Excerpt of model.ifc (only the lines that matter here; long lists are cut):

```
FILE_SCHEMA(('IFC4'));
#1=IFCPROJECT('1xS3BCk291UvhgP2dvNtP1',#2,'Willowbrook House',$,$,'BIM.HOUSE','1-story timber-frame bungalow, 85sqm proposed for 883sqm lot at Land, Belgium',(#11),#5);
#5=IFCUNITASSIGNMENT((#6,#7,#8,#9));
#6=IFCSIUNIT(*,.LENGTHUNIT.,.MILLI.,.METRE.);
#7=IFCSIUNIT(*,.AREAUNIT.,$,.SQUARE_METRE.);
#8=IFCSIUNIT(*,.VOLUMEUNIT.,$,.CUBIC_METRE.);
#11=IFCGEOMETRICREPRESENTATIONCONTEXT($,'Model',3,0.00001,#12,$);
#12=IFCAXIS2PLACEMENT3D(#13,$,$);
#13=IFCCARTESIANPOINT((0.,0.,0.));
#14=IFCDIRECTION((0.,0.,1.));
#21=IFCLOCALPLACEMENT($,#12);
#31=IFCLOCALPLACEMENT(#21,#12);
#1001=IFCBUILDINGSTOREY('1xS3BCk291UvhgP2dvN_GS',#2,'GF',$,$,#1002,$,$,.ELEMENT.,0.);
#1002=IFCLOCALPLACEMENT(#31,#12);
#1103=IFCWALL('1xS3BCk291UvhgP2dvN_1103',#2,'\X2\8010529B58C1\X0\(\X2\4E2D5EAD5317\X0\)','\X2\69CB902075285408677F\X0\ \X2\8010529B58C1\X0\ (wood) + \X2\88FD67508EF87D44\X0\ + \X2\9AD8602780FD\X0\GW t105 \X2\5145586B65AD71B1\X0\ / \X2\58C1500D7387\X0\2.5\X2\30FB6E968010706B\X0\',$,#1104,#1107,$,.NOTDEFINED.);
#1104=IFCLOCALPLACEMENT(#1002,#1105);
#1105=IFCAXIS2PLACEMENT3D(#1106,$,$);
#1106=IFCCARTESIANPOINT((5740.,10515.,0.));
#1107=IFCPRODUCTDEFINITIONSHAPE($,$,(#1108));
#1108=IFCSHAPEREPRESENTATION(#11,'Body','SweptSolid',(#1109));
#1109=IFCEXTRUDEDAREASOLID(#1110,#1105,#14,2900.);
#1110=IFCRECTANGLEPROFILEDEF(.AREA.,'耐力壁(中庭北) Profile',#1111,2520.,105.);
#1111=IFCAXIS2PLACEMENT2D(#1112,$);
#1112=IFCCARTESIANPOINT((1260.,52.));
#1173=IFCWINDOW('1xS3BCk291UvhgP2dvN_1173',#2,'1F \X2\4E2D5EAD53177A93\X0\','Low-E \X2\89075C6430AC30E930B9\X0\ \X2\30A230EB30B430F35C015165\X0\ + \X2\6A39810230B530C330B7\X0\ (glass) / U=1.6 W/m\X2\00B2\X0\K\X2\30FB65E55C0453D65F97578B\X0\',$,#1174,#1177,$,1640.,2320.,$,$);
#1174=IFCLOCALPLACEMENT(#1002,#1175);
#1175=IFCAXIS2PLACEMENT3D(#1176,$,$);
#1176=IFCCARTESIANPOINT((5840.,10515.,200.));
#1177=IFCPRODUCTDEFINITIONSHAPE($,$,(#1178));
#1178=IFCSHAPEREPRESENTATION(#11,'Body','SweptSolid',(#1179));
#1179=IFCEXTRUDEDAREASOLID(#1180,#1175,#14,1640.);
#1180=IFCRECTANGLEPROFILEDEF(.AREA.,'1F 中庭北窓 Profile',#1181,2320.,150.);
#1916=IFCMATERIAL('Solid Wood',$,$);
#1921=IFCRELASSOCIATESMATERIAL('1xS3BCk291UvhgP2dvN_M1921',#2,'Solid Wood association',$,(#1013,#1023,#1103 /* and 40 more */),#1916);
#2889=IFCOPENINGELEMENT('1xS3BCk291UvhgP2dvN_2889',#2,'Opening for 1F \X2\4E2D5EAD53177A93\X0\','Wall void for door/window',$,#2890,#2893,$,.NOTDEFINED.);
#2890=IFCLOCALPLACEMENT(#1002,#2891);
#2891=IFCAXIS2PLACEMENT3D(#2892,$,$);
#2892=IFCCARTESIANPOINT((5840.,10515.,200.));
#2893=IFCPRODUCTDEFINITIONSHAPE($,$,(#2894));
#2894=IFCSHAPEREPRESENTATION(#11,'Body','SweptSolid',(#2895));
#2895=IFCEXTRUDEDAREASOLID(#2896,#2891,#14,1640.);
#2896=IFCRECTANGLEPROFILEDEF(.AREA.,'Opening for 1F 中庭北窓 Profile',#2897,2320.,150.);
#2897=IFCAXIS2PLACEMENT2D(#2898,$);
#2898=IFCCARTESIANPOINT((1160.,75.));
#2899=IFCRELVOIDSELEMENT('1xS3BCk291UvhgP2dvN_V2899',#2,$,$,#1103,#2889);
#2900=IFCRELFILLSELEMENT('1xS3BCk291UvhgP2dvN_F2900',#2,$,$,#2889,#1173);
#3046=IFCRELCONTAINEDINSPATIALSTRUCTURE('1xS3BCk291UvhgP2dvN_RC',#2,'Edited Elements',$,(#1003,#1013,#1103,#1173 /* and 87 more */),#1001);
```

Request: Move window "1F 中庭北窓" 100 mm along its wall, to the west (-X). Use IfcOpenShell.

```python
import ifcopenshell
import ifcopenshell.api.geometry
import ifcopenshell.util.placement

model = ifcopenshell.open("model.ifc")

window = model.by_guid("1xS3BCk291UvhgP2dvN_1173")
opening = window.FillsVoids[0].RelatingOpeningElement
wall = opening.VoidsElements[0].RelatingBuildingElement

wall_matrix = ifcopenshell.util.placement.get_local_placement(wall.ObjectPlacement)
shift = wall_matrix[:3, 0] * -100.0
before = ifcopenshell.util.placement.get_local_placement(window.ObjectPlacement)[:3, 3].copy()

# The window is not placed relative to its opening, so move both.
for product in (opening, window):
    matrix = ifcopenshell.util.placement.get_local_placement(product.ObjectPlacement)
    matrix[:3, 3] += shift
    ifcopenshell.api.geometry.edit_object_placement(model, product=product, matrix=matrix, is_si=False)

after = ifcopenshell.util.placement.get_local_placement(window.ObjectPlacement)[:3, 3]
print("window moved by", (after - before).round(3) + 0.0)

model.write("model_edited.ifc")
```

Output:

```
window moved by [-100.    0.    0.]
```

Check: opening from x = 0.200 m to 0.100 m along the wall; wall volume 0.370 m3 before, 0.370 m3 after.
